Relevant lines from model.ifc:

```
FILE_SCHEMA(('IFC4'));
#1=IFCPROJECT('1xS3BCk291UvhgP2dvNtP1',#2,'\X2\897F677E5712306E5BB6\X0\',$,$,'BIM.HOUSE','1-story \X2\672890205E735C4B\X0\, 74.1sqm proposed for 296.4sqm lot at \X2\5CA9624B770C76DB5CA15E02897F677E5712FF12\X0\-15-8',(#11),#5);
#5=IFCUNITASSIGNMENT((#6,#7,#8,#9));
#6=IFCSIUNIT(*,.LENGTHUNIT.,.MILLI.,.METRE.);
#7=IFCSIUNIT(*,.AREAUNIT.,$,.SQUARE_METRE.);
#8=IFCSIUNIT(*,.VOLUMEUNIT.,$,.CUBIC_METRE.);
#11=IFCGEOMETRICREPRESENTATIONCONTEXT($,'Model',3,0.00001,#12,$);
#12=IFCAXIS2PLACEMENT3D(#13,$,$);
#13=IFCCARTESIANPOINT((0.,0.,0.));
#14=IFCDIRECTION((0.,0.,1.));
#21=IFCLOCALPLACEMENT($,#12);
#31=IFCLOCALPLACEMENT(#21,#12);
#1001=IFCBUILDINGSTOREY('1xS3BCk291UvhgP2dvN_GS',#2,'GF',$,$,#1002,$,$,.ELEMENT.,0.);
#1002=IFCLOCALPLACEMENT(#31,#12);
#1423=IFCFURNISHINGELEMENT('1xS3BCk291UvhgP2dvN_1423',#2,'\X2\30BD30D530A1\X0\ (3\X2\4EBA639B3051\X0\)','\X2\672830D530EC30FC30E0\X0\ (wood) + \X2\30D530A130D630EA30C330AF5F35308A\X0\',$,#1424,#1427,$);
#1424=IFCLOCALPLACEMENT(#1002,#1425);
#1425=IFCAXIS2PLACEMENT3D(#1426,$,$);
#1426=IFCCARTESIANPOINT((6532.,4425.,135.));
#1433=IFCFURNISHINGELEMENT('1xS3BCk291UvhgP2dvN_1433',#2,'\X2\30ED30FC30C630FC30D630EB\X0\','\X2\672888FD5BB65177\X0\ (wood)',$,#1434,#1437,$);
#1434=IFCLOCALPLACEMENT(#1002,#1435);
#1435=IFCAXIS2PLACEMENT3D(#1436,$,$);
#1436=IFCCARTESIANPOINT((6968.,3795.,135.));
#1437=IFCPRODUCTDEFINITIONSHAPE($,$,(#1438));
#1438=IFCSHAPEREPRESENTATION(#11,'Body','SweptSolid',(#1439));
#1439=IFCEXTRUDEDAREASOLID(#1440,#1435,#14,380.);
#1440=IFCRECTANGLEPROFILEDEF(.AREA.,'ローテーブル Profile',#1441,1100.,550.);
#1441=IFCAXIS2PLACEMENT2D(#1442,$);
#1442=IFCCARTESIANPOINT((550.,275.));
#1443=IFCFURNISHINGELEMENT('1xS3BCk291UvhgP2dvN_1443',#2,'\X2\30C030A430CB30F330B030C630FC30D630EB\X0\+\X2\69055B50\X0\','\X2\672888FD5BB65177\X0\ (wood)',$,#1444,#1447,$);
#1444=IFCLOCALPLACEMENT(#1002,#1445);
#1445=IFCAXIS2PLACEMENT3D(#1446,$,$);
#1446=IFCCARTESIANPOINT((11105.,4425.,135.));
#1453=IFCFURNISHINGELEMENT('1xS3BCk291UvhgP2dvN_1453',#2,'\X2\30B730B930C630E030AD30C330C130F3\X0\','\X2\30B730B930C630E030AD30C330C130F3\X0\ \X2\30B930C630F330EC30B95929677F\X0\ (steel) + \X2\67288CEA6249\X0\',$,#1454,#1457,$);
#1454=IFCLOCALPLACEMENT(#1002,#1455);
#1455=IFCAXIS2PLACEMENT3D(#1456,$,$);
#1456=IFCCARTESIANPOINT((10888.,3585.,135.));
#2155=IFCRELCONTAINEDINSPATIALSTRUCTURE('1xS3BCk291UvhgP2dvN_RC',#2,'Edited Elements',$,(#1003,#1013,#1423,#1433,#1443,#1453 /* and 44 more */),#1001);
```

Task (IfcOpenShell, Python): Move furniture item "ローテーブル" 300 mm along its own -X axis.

```python
import ifcopenshell
import ifcopenshell.api.geometry
import ifcopenshell.util.placement
import ifcopenshell.util.unit

model = ifcopenshell.open("model.ifc")
unit_scale = ifcopenshell.util.unit.calculate_unit_scale(model)

item = model.by_id(1433)
matrix = ifcopenshell.util.placement.get_local_placement(item.ObjectPlacement)
matrix[:3, 3] -= matrix[:3, 0] * 0.3 / unit_scale
ifcopenshell.api.geometry.edit_object_placement(model, product=item, matrix=matrix, is_si=False)

print(ifcopenshell.util.placement.get_local_placement(item.ObjectPlacement).round(3) + 0.0)

model.write("model_updated.ifc")
```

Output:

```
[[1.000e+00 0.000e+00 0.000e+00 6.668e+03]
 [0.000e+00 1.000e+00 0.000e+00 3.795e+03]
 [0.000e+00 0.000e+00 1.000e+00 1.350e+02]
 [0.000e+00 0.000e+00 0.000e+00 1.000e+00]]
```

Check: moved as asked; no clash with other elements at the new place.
